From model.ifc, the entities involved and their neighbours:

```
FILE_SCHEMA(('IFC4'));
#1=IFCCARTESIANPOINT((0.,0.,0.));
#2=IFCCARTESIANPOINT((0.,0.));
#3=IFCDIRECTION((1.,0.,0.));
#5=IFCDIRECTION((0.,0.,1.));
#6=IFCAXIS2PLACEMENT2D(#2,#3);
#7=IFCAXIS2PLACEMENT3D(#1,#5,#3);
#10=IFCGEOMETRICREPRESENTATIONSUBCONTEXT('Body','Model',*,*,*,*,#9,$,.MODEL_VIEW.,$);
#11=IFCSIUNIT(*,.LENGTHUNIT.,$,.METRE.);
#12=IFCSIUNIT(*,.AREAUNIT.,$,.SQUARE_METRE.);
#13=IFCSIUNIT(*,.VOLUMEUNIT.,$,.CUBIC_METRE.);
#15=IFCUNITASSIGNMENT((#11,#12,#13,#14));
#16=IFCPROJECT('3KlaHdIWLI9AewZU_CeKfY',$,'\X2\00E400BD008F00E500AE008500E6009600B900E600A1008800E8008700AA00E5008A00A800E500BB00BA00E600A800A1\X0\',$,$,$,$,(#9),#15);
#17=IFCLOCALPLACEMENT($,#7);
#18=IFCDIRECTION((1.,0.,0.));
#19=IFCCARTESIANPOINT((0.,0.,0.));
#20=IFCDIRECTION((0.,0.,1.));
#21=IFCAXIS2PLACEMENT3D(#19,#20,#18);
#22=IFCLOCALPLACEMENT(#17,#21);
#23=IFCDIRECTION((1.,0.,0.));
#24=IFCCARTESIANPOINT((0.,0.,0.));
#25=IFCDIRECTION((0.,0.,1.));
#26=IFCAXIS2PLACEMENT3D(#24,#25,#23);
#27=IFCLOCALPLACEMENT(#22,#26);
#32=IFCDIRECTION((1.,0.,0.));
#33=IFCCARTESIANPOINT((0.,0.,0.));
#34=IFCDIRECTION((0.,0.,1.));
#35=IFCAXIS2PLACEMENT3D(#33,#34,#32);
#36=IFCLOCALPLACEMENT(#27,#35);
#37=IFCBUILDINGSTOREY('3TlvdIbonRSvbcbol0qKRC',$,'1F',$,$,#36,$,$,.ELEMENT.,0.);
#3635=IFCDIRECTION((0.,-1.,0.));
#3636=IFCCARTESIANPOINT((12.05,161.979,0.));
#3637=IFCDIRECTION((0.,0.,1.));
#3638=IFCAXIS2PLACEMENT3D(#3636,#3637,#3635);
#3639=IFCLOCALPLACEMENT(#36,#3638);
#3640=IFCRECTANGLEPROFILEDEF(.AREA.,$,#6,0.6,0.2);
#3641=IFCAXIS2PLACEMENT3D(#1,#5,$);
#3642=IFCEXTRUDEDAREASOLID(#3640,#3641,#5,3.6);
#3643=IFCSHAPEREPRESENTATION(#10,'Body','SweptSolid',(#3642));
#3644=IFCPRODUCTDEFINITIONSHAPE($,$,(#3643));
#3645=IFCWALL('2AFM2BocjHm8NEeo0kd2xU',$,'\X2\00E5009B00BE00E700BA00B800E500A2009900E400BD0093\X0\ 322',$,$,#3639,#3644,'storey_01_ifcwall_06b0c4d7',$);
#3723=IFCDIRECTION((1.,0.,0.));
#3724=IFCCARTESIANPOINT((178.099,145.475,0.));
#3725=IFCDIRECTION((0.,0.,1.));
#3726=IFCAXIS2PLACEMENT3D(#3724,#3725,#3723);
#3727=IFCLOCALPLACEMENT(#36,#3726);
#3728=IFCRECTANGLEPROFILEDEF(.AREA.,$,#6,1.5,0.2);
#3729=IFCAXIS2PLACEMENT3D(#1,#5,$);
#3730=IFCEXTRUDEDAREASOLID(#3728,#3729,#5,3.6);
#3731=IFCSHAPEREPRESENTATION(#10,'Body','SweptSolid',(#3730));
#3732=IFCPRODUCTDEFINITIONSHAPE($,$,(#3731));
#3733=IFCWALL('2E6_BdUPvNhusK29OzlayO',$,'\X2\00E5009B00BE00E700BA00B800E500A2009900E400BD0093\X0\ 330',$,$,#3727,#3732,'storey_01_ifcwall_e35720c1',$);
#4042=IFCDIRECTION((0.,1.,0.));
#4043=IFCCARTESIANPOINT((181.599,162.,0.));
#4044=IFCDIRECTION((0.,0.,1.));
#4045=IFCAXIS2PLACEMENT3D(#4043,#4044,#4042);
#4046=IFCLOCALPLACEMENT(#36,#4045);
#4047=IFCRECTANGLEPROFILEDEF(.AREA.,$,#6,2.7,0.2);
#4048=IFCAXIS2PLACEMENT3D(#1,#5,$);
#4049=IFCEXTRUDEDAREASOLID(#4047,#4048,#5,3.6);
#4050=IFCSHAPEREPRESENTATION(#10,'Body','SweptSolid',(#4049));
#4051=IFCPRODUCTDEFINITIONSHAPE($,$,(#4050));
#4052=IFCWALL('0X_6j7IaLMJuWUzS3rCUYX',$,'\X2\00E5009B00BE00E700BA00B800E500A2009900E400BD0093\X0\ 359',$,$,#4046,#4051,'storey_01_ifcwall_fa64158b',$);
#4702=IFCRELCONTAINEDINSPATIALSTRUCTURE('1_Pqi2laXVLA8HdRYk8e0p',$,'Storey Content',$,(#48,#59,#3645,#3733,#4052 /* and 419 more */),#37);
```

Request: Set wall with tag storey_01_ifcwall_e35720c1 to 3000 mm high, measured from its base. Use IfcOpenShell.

```python
import ifcopenshell
import ifcopenshell.geom
import ifcopenshell.util.representation
import ifcopenshell.util.shape

model = ifcopenshell.open("model.ifc")
settings = ifcopenshell.geom.settings()


def volume(element):
    """Net volume in cubic metres, openings subtracted."""
    shape = ifcopenshell.geom.create_shape(settings, element)
    return ifcopenshell.util.shape.get_volume(shape.geometry)


wall = model.by_guid("2E6_BdUPvNhusK29OzlayO")
before = volume(wall)

body = ifcopenshell.util.representation.get_representation(wall, "Model", "Body")
solid = body.Items[0]
old_height = solid.Depth
solid.Depth = 3.0
after = volume(wall)

print(f"height {old_height:g} -> {solid.Depth:g}, volume {before:.3f} -> {after:.3f} m3")

model.write("model_updated.ifc")
```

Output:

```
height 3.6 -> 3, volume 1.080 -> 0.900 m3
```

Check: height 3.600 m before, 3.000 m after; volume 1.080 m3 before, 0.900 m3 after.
